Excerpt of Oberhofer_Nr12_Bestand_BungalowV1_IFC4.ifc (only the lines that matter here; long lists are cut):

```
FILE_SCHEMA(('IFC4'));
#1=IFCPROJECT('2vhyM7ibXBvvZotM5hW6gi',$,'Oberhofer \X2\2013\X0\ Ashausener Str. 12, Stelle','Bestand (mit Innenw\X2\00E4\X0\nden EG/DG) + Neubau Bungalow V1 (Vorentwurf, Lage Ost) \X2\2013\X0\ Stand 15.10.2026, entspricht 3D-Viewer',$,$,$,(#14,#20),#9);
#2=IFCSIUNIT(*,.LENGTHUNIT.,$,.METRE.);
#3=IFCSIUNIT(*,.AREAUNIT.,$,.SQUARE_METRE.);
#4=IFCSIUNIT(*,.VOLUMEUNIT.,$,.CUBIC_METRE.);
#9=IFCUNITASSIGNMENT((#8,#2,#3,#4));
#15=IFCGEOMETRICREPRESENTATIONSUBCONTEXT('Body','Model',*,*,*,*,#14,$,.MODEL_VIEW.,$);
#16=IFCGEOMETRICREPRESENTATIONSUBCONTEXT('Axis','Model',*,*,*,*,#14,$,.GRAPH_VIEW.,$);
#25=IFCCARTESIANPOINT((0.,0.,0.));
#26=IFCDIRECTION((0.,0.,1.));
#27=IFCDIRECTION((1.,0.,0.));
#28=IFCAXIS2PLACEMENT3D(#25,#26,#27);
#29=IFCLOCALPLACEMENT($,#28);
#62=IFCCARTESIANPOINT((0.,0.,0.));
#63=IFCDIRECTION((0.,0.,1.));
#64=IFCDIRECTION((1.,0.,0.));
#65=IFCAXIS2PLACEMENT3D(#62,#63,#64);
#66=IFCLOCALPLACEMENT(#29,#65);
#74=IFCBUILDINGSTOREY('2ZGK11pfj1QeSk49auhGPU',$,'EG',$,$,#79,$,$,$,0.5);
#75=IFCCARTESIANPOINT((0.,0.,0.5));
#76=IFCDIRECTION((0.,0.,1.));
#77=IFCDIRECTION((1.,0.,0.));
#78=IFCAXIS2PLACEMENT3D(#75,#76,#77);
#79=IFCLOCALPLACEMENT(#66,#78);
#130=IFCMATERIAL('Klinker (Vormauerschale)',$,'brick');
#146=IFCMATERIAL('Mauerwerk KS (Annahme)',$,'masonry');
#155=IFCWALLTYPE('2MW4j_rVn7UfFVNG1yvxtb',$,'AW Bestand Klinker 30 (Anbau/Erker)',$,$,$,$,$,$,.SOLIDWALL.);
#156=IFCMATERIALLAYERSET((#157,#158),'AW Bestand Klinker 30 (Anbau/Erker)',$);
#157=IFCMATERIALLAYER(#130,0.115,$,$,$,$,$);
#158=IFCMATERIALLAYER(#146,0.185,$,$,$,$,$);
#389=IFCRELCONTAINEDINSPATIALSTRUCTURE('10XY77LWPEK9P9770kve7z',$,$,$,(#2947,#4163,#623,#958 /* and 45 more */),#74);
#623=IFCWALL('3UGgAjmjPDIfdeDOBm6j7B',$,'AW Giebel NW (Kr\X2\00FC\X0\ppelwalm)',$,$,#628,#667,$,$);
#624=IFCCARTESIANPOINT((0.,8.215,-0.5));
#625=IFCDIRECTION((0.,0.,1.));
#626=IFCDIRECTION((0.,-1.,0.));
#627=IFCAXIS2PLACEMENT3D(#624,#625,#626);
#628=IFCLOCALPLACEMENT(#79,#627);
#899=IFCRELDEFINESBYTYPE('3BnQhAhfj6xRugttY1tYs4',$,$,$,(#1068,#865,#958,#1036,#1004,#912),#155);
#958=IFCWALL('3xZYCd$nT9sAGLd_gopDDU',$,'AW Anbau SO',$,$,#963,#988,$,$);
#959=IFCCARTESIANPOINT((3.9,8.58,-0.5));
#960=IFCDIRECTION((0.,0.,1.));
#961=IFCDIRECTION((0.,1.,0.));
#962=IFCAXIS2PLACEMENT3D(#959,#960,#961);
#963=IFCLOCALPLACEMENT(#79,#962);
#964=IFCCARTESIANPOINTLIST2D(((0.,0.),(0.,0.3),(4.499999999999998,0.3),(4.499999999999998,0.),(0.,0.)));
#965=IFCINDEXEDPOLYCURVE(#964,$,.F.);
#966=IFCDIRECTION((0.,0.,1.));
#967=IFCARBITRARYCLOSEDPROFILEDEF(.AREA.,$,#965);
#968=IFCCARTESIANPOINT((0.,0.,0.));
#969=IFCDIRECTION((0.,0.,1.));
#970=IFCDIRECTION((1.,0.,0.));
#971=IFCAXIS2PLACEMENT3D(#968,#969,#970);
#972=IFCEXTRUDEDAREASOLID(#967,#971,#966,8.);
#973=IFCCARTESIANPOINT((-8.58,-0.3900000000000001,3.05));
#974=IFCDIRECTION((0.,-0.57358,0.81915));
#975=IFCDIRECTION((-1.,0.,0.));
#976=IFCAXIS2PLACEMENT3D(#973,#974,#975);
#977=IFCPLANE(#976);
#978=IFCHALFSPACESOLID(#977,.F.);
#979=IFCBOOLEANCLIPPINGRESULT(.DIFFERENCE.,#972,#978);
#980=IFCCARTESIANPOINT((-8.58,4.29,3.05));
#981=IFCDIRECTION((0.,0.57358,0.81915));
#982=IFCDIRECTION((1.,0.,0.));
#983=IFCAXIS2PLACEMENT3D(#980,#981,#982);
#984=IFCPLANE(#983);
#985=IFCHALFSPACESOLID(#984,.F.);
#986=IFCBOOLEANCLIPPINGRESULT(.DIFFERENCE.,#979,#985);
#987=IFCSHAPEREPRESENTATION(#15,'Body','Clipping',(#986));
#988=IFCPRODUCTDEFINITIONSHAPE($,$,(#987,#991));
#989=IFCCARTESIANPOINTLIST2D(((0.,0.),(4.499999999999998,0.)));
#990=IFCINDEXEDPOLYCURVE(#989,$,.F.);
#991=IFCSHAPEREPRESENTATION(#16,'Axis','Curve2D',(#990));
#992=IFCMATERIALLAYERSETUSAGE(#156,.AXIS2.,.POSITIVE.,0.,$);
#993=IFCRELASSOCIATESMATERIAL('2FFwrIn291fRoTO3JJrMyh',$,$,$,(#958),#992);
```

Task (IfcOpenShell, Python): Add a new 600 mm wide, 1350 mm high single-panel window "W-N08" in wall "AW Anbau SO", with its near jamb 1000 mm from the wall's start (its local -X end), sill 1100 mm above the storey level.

```python
import numpy as np
import ifcopenshell
import ifcopenshell.api.feature
import ifcopenshell.api.geometry
import ifcopenshell.api.root
import ifcopenshell.api.spatial
import ifcopenshell.geom
import ifcopenshell.util.element
import ifcopenshell.util.placement
import ifcopenshell.util.representation
import ifcopenshell.util.shape
import ifcopenshell.util.unit

model = ifcopenshell.open("Oberhofer_Nr12_Bestand_BungalowV1_IFC4.ifc")
unit_scale = ifcopenshell.util.unit.calculate_unit_scale(model)
settings = ifcopenshell.geom.settings()


def volume(element):
    """Net volume in cubic metres, openings subtracted."""
    shape = ifcopenshell.geom.create_shape(settings, element)
    return ifcopenshell.util.shape.get_volume(shape.geometry)


wall = model.by_guid("3xZYCd$nT9sAGLd_gopDDU")
storey = ifcopenshell.util.element.get_container(wall, ifc_class="IfcBuildingStorey")
context = ifcopenshell.util.representation.get_context(model, "Model", "Body", "MODEL_VIEW")
before = volume(wall)

width, height, from_end, sill = 0.6, 1.35, 1, 1.1  # metres

# The wall runs along its own X axis, and the end named is its -X end.
wall_shape = ifcopenshell.geom.create_shape(settings, wall)
x, y, z = ifcopenshell.util.shape.get_vertices(wall_shape.geometry).T
start = x.min() + from_end
face, thickness = float(y.min()), float(y.max() - y.min())
wall_matrix = ifcopenshell.util.placement.get_local_placement(wall.ObjectPlacement)
level = ifcopenshell.util.placement.get_local_placement(storey.ObjectPlacement)[2, 3]


def in_wall(x, y):
    """Placement at x, y metres in the wall's axes, at sill height."""
    matrix = wall_matrix.copy()
    matrix[:, 3] = wall_matrix @ np.array([x / unit_scale, y / unit_scale, 0.0, 1.0])
    matrix[2, 3] = level + sill / unit_scale
    return matrix


# Opening: a box that overshoots both wall faces by 50 mm.
opening = ifcopenshell.api.root.create_entity(model, ifc_class="IfcOpeningElement", predefined_type="OPENING")
box = ifcopenshell.api.geometry.add_wall_representation(
    model, context=context, length=width, height=height, thickness=thickness + 0.1
)
ifcopenshell.api.geometry.assign_representation(model, product=opening, representation=box)
ifcopenshell.api.geometry.edit_object_placement(model, product=opening, matrix=in_wall(start, face - 0.05), is_si=False)
ifcopenshell.api.feature.add_feature(model, feature=opening, element=wall)

window = ifcopenshell.api.root.create_entity(model, ifc_class="IfcWindow", name="W-N08", predefined_type="WINDOW")
window.OverallWidth, window.OverallHeight = width / unit_scale, height / unit_scale
window.PartitioningType = "SINGLE_PANEL"
body = ifcopenshell.api.geometry.add_window_representation(
    model,
    context=context,
    overall_width=window.OverallWidth,
    overall_height=window.OverallHeight,
    partition_type="SINGLE_PANEL",
)
ifcopenshell.api.geometry.assign_representation(model, product=window, representation=body)
ifcopenshell.api.spatial.assign_container(model, products=[window], relating_structure=storey)
ifcopenshell.api.feature.add_filling(model, opening=opening, element=window)

# Centre the window in the wall's thickness.
ifcopenshell.api.geometry.edit_object_placement(model, product=window, matrix=in_wall(start, face), is_si=False)
window_shape = ifcopenshell.geom.create_shape(settings, window)
depth = ifcopenshell.util.shape.get_vertices(window_shape.geometry)[:, 1]
offset = face + thickness / 2 - (depth.min() + depth.max()) / 2
ifcopenshell.api.geometry.edit_object_placement(model, product=window, matrix=in_wall(start, offset), is_si=False)

after = volume(wall)

print(f"wall volume {before:.3f} -> {after:.3f} m3")

model.write("Oberhofer_Nr12_Bestand_BungalowV1_IFC4_edited.ifc")
```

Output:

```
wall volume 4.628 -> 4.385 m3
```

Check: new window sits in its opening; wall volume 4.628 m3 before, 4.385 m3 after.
